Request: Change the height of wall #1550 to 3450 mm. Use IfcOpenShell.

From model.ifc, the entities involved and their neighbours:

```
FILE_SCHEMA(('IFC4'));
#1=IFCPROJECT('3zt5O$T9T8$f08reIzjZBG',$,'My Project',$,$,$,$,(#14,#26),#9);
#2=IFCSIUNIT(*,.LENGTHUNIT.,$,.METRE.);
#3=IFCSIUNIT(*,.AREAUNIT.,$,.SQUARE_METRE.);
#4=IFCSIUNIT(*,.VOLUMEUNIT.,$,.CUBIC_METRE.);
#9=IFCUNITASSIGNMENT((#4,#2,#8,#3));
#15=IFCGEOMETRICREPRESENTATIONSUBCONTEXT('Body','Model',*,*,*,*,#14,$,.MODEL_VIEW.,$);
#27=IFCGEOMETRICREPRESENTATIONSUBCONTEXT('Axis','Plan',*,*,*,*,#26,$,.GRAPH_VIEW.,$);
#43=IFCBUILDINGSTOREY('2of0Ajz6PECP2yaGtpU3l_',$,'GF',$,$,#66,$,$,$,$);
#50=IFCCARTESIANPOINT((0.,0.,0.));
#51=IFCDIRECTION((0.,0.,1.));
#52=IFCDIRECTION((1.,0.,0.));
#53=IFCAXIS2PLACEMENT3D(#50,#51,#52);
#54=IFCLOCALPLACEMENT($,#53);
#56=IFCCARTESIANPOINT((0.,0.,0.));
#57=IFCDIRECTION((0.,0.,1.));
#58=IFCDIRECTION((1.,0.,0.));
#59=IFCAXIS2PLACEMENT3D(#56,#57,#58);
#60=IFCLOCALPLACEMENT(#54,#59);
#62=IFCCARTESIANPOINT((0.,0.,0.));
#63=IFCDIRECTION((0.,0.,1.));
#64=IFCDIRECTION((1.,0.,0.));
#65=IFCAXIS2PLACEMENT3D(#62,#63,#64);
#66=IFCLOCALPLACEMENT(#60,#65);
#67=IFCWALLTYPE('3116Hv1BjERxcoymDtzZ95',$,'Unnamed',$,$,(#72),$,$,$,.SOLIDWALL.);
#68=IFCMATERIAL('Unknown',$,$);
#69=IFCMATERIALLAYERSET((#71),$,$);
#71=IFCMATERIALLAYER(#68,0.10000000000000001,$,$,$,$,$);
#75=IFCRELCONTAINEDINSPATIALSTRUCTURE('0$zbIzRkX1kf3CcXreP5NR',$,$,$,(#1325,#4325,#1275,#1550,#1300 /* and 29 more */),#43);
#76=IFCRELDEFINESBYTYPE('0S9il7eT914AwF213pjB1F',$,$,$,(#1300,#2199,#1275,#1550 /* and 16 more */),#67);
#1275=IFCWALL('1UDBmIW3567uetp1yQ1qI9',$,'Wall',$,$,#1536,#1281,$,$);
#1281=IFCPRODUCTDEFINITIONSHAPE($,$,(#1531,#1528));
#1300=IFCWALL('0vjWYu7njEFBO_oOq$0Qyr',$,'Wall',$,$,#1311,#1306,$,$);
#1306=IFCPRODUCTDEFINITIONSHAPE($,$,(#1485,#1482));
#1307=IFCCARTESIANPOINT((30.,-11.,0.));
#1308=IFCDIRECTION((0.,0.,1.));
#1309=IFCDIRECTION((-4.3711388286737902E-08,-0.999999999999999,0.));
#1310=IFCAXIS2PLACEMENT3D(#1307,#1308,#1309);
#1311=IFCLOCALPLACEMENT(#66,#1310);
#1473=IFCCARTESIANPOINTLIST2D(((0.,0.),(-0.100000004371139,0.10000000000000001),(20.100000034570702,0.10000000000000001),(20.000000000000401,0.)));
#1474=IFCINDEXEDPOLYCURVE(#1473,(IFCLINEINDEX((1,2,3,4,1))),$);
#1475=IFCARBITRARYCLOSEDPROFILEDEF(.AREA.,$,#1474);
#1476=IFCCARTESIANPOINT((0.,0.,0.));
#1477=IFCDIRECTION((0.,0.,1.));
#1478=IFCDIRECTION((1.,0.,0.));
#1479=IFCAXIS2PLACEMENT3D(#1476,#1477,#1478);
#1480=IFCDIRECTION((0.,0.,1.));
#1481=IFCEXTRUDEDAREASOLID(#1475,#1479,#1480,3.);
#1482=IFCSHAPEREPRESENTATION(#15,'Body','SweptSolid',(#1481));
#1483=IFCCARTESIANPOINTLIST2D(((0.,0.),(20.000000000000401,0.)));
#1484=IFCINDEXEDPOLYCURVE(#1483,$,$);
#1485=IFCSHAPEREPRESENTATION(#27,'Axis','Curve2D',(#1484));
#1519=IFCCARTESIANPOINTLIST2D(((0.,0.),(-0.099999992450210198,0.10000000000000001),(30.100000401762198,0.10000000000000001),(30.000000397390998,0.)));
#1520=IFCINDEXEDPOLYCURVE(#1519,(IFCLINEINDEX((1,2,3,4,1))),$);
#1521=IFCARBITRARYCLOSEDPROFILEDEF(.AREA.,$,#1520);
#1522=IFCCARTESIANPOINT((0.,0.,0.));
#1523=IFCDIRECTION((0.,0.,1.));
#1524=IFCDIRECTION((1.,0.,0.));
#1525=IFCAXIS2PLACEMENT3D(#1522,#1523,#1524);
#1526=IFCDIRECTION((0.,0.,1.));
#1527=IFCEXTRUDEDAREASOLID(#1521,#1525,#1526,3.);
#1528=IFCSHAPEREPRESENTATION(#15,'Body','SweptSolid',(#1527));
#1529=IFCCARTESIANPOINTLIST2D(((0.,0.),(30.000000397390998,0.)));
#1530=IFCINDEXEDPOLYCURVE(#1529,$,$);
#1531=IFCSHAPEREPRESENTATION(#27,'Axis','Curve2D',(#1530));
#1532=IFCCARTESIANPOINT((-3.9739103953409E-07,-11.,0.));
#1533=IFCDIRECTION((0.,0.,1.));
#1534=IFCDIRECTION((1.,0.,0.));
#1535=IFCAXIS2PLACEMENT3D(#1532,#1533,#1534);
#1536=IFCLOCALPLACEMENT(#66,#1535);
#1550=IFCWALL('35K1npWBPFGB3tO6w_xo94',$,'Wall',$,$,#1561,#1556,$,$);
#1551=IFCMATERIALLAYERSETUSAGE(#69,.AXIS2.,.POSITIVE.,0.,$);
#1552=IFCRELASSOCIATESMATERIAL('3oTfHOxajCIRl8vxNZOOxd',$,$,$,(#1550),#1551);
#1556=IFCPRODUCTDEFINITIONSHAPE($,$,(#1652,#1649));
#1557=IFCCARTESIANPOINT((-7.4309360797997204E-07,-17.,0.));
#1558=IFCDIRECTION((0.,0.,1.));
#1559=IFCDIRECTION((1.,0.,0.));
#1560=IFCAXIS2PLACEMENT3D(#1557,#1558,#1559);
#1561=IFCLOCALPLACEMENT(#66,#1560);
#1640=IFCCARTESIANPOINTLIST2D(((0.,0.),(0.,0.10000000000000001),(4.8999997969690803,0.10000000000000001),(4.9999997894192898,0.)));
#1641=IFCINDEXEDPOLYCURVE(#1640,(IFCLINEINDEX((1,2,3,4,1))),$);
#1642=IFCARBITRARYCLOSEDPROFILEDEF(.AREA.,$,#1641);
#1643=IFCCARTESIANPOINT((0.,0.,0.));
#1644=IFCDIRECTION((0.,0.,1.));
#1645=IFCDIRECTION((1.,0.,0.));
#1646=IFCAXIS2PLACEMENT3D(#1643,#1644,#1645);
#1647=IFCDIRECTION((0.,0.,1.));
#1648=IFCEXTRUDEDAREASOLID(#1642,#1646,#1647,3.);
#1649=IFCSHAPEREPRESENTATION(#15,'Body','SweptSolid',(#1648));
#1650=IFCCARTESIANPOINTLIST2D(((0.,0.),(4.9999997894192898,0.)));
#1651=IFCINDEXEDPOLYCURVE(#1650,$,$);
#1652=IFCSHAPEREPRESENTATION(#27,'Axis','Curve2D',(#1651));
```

```python
import ifcopenshell
import ifcopenshell.geom
import ifcopenshell.util.representation
import ifcopenshell.util.shape

model = ifcopenshell.open("model.ifc")
settings = ifcopenshell.geom.settings()


def volume(element):
    """Net volume in cubic metres, openings subtracted."""
    shape = ifcopenshell.geom.create_shape(settings, element)
    return ifcopenshell.util.shape.get_volume(shape.geometry)


wall = model.by_guid("35K1npWBPFGB3tO6w_xo94")
before = volume(wall)

body = ifcopenshell.util.representation.get_representation(wall, "Model", "Body")
solid = body.Items[0]
old_height = solid.Depth
solid.Depth = 3.45
after = volume(wall)

print(f"height {old_height:g} -> {solid.Depth:g}, volume {before:.3f} -> {after:.3f} m3")

model.write("model_rev.ifc")
```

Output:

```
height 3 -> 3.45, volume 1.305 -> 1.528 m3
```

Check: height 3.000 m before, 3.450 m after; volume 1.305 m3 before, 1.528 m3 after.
